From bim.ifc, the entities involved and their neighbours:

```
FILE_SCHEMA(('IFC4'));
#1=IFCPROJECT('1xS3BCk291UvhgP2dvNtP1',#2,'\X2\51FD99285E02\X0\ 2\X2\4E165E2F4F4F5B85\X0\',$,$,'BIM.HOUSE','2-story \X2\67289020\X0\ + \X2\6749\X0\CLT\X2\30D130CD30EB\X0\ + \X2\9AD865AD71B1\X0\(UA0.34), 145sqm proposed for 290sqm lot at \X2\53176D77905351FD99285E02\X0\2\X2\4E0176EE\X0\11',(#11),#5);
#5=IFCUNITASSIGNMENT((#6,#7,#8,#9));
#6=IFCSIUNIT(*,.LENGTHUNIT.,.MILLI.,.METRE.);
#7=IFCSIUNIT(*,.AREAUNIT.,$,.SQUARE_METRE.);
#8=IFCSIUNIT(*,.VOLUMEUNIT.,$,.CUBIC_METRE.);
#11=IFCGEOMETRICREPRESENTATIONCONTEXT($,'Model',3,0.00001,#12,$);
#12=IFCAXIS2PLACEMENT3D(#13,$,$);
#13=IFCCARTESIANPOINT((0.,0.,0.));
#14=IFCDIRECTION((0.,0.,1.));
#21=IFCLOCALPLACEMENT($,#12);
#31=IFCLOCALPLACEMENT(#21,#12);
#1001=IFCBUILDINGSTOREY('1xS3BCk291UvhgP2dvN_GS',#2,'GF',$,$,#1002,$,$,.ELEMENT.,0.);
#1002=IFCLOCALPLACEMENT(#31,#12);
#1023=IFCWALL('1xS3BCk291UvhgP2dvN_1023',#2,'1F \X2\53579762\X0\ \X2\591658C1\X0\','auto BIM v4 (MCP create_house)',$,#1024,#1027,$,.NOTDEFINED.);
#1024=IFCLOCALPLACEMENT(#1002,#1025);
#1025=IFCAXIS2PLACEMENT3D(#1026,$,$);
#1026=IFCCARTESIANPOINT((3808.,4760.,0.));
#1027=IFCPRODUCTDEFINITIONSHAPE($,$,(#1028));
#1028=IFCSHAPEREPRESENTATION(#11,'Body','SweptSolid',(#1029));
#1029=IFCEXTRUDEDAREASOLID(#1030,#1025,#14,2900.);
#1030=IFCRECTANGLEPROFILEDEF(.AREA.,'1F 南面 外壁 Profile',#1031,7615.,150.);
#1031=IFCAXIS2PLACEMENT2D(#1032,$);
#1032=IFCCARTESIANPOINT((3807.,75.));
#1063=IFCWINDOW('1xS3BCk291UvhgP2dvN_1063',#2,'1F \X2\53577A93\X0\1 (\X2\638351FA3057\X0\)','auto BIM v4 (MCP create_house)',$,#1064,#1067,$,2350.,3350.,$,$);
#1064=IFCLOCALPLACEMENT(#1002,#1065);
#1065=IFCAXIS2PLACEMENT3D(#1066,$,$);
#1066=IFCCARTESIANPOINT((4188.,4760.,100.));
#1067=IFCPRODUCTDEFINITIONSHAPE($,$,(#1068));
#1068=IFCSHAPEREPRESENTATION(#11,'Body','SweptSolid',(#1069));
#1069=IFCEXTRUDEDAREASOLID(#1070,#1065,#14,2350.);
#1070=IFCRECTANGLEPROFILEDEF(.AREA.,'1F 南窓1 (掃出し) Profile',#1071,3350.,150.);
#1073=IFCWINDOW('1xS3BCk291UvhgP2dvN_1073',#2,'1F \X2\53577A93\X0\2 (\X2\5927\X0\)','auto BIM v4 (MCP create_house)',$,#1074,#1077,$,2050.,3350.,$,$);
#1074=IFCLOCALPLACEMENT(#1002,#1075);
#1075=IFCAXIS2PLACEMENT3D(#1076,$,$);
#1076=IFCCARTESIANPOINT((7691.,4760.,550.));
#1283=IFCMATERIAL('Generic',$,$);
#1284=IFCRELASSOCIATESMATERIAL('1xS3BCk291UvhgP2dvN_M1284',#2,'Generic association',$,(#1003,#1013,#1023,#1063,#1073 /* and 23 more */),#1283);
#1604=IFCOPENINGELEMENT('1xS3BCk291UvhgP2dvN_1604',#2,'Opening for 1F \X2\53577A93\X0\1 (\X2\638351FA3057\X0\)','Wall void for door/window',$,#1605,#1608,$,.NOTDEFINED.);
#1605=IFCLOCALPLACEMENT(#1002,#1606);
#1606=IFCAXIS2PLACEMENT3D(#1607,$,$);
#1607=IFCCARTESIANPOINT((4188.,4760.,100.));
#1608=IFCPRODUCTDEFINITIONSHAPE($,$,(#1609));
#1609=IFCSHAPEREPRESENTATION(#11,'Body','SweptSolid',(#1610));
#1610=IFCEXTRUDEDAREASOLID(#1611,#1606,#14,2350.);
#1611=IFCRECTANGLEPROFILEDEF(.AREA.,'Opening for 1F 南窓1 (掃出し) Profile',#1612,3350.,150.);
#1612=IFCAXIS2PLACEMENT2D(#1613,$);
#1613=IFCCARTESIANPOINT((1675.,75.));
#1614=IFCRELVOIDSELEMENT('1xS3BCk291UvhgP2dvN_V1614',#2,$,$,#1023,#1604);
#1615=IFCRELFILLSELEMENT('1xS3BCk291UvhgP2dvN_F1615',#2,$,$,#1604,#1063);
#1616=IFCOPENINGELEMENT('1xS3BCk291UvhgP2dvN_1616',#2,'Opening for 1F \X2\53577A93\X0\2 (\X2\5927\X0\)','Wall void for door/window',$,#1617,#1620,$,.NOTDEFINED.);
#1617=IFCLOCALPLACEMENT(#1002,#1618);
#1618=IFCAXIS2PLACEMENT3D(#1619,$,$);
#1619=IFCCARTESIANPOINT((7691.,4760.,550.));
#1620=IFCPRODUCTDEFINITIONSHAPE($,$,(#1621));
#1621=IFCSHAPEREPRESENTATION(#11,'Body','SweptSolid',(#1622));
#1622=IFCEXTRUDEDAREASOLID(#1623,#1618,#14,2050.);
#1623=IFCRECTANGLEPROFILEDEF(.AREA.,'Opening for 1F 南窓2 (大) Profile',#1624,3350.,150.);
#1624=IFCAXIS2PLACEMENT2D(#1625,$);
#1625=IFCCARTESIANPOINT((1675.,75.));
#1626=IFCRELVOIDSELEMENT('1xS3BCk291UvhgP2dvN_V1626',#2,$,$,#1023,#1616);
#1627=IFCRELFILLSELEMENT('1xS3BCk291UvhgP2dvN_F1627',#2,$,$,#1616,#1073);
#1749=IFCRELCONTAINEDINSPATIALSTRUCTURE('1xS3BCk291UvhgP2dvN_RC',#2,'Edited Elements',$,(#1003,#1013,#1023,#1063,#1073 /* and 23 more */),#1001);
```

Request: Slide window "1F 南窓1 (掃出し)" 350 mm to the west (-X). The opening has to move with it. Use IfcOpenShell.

```python
import ifcopenshell
import ifcopenshell.api.geometry
import ifcopenshell.util.placement

model = ifcopenshell.open("bim.ifc")

window = model.by_guid("1xS3BCk291UvhgP2dvN_1063")
opening = window.FillsVoids[0].RelatingOpeningElement
wall = opening.VoidsElements[0].RelatingBuildingElement

wall_matrix = ifcopenshell.util.placement.get_local_placement(wall.ObjectPlacement)
shift = wall_matrix[:3, 0] * -350.0
before = ifcopenshell.util.placement.get_local_placement(window.ObjectPlacement)[:3, 3].copy()

# The window is not placed relative to its opening, so move both.
for product in (opening, window):
    matrix = ifcopenshell.util.placement.get_local_placement(product.ObjectPlacement)
    matrix[:3, 3] += shift
    ifcopenshell.api.geometry.edit_object_placement(model, product=product, matrix=matrix, is_si=False)

after = ifcopenshell.util.placement.get_local_placement(window.ObjectPlacement)[:3, 3]
print("window moved by", (after - before).round(3) + 0.0)

model.write("bim_edited.ifc")
```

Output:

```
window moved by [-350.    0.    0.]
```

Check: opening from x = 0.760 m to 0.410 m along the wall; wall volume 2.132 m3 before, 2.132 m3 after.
